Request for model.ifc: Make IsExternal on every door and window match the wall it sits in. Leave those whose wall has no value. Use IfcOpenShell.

First a look at what the model holds.

```python
import ifcopenshell
import ifcopenshell.util.element

model = ifcopenshell.open("model.ifc")
print(model.schema)
seen = {}
for e in model.by_type("IfcDoor") + model.by_type("IfcWindow"):
    if not e.FillsVoids:
        continue
    host = e.FillsVoids[0].RelatingOpeningElement.VoidsElements[0].RelatingBuildingElement
    own = ifcopenshell.util.element.get_pset(e, f"Pset_{e.is_a()[3:].removesuffix('StandardCase')}Common", "IsExternal")
    wall = ifcopenshell.util.element.get_pset(host, "Pset_WallCommon", "IsExternal")
    seen[e.is_a(), own, wall] = seen.get((e.is_a(), own, wall), 0) + 1
for (cls, own, wall), count in sorted(seen.items(), key=str):
    print(count, cls, "IsExternal:", own, "| host wall:", wall)
```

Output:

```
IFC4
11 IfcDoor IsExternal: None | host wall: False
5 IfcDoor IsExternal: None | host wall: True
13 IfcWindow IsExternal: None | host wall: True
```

```python
import ifcopenshell
import ifcopenshell.api.pset
import ifcopenshell.util.element

model = ifcopenshell.open("model.ifc")

count = 0
for ifc_class, pset_name in (("IfcDoor", "Pset_DoorCommon"), ("IfcWindow", "Pset_WindowCommon")):
    for e in model.by_type(ifc_class):
        if not e.FillsVoids:
            continue
        host = e.FillsVoids[0].RelatingOpeningElement.VoidsElements[0].RelatingBuildingElement
        external = ifcopenshell.util.element.get_pset(host, "Pset_WallCommon", "IsExternal")
        if external is None or ifcopenshell.util.element.get_pset(e, pset_name, "IsExternal") == external:
            continue
        pset = ifcopenshell.api.pset.add_pset(model, product=e, name=pset_name)
        ifcopenshell.api.pset.edit_pset(model, pset=pset, properties={"IsExternal": external})
        count += 1

print(count, "updated")

model.write("model_edited.ifc")
```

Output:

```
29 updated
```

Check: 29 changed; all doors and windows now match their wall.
